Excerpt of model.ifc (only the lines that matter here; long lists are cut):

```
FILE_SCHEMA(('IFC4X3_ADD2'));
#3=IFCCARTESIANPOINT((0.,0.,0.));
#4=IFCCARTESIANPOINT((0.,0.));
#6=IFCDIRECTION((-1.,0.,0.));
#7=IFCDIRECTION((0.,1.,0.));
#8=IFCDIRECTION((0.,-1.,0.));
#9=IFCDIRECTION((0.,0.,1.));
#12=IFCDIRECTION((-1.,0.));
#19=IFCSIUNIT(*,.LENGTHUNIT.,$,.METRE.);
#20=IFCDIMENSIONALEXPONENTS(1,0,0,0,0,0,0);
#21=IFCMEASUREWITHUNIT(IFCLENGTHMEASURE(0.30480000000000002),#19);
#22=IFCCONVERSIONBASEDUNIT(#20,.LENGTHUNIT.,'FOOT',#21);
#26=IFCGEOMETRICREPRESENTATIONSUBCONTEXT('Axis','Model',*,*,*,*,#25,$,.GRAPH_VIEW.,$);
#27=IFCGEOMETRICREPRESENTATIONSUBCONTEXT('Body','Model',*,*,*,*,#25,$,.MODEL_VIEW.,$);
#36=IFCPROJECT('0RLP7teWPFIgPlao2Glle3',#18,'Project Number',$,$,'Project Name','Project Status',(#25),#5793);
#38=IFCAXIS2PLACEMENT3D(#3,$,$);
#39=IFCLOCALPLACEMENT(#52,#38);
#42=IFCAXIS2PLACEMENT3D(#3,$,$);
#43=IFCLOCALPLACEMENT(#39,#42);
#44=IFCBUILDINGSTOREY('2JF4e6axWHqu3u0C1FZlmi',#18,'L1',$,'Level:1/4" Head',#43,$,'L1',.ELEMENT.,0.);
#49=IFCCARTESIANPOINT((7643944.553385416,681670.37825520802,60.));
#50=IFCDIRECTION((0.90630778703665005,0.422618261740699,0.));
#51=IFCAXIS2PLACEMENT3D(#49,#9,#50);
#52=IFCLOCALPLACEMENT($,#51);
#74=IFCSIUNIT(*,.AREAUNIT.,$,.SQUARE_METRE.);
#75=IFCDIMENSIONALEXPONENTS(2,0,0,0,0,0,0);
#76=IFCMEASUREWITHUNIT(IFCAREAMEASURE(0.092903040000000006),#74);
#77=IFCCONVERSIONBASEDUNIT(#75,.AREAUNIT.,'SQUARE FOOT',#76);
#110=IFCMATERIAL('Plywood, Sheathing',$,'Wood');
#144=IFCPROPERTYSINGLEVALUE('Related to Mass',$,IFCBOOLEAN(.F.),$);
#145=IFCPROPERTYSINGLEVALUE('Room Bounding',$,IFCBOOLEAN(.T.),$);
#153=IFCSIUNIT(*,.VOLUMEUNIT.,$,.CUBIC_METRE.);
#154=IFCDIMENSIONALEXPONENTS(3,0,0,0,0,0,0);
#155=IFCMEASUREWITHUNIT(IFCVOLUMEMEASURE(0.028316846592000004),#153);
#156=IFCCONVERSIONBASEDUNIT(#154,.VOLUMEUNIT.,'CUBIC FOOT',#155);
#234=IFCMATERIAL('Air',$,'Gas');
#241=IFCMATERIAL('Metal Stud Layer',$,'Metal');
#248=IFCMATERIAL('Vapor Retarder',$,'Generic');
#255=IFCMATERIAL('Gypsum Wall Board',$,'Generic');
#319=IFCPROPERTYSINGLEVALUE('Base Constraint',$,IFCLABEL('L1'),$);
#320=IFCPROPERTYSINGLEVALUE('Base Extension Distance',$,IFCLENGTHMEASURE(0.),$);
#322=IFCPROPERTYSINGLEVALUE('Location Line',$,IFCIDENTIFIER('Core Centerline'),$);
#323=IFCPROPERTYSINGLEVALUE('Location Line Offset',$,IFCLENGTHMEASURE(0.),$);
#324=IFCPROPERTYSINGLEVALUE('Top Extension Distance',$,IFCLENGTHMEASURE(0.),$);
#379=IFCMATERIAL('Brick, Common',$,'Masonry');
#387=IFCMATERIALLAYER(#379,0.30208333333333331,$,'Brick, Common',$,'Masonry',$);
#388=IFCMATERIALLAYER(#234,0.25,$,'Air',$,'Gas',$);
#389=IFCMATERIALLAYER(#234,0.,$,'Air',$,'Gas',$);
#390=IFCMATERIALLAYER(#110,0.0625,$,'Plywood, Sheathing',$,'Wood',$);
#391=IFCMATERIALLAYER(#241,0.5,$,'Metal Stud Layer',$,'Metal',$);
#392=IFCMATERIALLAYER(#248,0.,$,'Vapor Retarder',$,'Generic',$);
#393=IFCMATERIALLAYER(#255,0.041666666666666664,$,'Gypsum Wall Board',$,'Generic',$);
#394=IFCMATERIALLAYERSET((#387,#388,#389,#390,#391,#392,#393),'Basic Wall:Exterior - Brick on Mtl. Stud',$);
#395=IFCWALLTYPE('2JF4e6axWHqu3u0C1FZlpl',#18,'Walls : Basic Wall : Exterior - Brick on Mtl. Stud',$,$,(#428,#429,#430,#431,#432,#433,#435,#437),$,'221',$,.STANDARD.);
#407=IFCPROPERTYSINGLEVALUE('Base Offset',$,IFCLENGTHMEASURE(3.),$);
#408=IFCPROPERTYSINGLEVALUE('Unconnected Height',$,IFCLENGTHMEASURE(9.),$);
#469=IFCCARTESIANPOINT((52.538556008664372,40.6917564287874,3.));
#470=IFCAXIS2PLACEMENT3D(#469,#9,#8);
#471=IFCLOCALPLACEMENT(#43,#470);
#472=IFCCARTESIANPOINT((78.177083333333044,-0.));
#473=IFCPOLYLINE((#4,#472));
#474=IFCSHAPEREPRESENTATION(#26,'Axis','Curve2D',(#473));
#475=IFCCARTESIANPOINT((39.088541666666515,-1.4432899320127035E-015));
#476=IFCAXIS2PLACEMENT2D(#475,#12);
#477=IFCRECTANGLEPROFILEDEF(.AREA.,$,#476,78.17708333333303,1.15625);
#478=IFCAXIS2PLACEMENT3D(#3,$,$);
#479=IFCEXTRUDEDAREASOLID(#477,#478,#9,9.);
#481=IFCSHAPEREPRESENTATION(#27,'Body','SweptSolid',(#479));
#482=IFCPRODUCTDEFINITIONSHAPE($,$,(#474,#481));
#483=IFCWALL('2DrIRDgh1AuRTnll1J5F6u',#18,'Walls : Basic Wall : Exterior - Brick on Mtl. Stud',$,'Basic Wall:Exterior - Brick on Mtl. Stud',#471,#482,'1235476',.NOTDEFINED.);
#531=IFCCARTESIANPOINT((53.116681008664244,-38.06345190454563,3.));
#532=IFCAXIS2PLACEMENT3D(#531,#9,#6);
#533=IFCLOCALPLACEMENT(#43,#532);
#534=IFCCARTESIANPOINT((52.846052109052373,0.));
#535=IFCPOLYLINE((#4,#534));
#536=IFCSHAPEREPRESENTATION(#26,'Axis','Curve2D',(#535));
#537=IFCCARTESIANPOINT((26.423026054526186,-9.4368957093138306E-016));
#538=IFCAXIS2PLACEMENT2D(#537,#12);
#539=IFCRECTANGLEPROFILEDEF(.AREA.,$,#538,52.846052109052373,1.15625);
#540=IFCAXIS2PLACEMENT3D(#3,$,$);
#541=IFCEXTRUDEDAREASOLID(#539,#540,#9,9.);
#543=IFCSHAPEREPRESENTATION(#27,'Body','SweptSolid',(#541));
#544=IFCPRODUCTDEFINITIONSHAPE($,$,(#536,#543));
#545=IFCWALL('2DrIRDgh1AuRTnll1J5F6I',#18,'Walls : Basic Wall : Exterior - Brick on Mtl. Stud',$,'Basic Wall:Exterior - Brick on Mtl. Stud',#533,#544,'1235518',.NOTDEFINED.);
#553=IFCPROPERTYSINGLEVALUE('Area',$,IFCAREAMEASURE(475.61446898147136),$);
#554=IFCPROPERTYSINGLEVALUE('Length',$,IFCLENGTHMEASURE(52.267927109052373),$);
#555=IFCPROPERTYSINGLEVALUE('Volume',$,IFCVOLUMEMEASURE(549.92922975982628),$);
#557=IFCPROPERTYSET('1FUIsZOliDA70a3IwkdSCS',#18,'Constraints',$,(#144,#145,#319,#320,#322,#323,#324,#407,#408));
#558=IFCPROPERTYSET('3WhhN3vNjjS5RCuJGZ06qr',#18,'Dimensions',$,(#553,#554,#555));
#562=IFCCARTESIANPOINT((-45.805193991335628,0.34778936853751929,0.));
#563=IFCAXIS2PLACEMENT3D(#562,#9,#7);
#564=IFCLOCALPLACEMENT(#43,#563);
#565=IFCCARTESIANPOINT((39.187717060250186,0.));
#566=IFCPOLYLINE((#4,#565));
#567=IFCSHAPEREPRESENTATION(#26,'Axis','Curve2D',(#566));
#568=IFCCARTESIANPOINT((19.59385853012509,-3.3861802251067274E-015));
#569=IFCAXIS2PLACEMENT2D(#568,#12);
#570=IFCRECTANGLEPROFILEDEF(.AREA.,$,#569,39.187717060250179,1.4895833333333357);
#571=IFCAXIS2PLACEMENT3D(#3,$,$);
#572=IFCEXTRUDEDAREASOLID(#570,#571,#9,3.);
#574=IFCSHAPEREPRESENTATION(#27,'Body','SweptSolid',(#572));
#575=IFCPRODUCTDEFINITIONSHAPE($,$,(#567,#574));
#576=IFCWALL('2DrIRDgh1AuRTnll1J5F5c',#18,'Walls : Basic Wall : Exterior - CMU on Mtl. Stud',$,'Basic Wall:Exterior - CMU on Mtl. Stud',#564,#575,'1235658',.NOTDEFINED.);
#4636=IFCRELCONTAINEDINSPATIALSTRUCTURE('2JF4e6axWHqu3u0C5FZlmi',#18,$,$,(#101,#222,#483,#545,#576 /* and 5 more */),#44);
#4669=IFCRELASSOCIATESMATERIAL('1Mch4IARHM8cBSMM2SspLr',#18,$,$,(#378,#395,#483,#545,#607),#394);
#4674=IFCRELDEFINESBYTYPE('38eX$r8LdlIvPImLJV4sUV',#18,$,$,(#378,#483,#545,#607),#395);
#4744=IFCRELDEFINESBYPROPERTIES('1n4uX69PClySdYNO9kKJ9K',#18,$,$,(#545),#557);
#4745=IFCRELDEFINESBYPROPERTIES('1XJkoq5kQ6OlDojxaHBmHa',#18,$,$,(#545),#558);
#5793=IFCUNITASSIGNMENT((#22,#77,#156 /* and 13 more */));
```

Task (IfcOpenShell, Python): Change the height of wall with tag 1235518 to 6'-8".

```python
import ifcopenshell
import ifcopenshell.api.pset
import ifcopenshell.geom
import ifcopenshell.util.element
import ifcopenshell.util.representation
import ifcopenshell.util.shape
import ifcopenshell.util.unit

model = ifcopenshell.open("model.ifc")
unit_scale = ifcopenshell.util.unit.calculate_unit_scale(model)
area_scale = ifcopenshell.util.unit.calculate_unit_scale(model, "AREAUNIT")
volume_scale = ifcopenshell.util.unit.calculate_unit_scale(model, "VOLUMEUNIT")
settings = ifcopenshell.geom.settings()


def volume(element):
    """Net volume in cubic metres, openings subtracted."""
    shape = ifcopenshell.geom.create_shape(settings, element)
    return ifcopenshell.util.shape.get_volume(shape.geometry)


wall = model.by_guid("2DrIRDgh1AuRTnll1J5F6I")
before = volume(wall)

body = ifcopenshell.util.representation.get_representation(wall, "Model", "Body")
solid = body.Items[0]
old_height = solid.Depth
solid.Depth = 80 * 0.0254 / unit_scale
after = volume(wall)
thickness = 0.3524  # wall thickness in metres

# Update the stored height, areas and volumes.
pset = model.by_id(ifcopenshell.util.element.get_pset(wall, "Constraints", should_inherit=False)["id"])
ifcopenshell.api.pset.edit_pset(model, pset=pset, properties={
    "Unconnected Height": model.create_entity("IfcLengthMeasure", solid.Depth),
})
pset = model.by_id(ifcopenshell.util.element.get_pset(wall, "Dimensions", should_inherit=False)["id"])
ifcopenshell.api.pset.edit_pset(model, pset=pset, properties={
    "Area": model.create_entity("IfcAreaMeasure", after / thickness / area_scale),
    "Volume": model.create_entity("IfcVolumeMeasure", after / volume_scale),
})

print(f"height {old_height:g} -> {solid.Depth:g}, volume {before:.3f} -> {after:.3f} m3")

model.write("model-out.ifc")
```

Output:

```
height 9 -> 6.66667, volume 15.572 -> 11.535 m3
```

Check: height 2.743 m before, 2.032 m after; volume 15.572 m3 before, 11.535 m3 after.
